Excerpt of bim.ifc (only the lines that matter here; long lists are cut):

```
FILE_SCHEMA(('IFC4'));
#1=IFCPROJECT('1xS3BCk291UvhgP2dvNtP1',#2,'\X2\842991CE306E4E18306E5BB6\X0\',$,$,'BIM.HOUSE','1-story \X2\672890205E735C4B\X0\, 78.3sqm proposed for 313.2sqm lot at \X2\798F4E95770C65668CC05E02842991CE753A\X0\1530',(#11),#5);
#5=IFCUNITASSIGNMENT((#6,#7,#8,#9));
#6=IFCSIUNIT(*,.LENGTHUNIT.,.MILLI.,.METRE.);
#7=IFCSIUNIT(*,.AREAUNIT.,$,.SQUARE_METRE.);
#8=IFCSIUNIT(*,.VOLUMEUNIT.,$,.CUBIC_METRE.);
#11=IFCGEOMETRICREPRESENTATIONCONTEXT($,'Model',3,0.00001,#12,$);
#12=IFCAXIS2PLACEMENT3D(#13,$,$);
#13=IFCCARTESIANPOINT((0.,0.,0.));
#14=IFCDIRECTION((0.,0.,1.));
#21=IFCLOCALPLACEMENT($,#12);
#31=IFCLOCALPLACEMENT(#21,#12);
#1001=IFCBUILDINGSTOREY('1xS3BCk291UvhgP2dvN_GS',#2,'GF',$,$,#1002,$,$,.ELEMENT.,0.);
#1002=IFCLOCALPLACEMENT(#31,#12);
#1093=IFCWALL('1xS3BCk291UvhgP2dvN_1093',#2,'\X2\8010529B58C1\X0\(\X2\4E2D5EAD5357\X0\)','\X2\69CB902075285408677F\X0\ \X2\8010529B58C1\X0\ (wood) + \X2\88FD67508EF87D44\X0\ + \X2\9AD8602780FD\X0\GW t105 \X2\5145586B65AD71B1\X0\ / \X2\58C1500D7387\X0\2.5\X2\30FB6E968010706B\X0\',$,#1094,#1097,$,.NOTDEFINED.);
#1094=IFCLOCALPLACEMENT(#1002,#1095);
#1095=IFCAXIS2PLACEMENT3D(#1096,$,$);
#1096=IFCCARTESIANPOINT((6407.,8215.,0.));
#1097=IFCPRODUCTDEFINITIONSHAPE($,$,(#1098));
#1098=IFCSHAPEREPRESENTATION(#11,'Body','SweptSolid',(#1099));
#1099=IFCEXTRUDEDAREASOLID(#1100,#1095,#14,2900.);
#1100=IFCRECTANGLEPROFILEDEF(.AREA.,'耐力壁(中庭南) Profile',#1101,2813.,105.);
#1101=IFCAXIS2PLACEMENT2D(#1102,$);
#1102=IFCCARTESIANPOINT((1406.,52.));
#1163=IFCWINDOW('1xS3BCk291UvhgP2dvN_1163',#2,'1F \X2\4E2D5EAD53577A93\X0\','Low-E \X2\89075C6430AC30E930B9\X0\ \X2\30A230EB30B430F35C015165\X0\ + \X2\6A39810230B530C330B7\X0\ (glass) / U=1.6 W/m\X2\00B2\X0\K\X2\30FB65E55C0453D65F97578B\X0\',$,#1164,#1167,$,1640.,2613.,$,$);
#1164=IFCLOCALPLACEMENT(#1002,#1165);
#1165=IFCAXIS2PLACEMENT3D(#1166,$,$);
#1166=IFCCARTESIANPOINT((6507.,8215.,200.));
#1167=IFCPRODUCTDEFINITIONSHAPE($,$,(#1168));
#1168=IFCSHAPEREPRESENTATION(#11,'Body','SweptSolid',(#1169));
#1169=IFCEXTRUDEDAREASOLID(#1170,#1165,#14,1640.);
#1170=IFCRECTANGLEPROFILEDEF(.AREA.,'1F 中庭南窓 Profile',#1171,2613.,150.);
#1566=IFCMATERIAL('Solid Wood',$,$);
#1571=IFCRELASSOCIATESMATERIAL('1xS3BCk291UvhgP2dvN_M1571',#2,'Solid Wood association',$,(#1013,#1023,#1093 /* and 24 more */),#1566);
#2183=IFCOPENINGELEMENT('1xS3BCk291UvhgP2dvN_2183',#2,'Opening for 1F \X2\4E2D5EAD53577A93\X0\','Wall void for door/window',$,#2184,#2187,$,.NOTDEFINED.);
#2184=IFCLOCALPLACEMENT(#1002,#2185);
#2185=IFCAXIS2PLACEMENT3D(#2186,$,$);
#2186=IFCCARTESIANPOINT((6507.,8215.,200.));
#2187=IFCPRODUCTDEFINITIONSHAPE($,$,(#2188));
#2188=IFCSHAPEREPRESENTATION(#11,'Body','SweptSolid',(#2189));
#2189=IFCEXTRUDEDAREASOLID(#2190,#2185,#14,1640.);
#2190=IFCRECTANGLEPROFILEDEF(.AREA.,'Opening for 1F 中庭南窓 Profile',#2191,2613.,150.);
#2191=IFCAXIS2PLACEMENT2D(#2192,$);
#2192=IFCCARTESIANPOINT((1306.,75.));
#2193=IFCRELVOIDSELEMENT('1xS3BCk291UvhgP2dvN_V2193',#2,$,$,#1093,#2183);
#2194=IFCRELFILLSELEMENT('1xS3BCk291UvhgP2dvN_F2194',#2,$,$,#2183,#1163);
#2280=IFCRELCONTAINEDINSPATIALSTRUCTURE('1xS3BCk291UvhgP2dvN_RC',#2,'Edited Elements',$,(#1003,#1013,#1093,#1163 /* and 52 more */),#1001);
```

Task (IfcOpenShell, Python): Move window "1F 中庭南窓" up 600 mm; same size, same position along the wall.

```python
import numpy as np
import ifcopenshell
import ifcopenshell.api.geometry
import ifcopenshell.util.placement
import ifcopenshell.util.unit

model = ifcopenshell.open("bim.ifc")
unit_scale = ifcopenshell.util.unit.calculate_unit_scale(model)

window = model.by_guid("1xS3BCk291UvhgP2dvN_1163")
opening = window.FillsVoids[0].RelatingOpeningElement
dz = 600.0

shift = np.array([0.0, 0.0, dz])
# The window is not placed relative to its opening, so move both.
for product in (opening, window):
    matrix = ifcopenshell.util.placement.get_local_placement(product.ObjectPlacement)
    matrix[:3, 3] += shift
    ifcopenshell.api.geometry.edit_object_placement(model, product=product, matrix=matrix, is_si=False)

print(f"moved by {dz * unit_scale:+.3f} m")

model.write("bim_rev.ifc")
```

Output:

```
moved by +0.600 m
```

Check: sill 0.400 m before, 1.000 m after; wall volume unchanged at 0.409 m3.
